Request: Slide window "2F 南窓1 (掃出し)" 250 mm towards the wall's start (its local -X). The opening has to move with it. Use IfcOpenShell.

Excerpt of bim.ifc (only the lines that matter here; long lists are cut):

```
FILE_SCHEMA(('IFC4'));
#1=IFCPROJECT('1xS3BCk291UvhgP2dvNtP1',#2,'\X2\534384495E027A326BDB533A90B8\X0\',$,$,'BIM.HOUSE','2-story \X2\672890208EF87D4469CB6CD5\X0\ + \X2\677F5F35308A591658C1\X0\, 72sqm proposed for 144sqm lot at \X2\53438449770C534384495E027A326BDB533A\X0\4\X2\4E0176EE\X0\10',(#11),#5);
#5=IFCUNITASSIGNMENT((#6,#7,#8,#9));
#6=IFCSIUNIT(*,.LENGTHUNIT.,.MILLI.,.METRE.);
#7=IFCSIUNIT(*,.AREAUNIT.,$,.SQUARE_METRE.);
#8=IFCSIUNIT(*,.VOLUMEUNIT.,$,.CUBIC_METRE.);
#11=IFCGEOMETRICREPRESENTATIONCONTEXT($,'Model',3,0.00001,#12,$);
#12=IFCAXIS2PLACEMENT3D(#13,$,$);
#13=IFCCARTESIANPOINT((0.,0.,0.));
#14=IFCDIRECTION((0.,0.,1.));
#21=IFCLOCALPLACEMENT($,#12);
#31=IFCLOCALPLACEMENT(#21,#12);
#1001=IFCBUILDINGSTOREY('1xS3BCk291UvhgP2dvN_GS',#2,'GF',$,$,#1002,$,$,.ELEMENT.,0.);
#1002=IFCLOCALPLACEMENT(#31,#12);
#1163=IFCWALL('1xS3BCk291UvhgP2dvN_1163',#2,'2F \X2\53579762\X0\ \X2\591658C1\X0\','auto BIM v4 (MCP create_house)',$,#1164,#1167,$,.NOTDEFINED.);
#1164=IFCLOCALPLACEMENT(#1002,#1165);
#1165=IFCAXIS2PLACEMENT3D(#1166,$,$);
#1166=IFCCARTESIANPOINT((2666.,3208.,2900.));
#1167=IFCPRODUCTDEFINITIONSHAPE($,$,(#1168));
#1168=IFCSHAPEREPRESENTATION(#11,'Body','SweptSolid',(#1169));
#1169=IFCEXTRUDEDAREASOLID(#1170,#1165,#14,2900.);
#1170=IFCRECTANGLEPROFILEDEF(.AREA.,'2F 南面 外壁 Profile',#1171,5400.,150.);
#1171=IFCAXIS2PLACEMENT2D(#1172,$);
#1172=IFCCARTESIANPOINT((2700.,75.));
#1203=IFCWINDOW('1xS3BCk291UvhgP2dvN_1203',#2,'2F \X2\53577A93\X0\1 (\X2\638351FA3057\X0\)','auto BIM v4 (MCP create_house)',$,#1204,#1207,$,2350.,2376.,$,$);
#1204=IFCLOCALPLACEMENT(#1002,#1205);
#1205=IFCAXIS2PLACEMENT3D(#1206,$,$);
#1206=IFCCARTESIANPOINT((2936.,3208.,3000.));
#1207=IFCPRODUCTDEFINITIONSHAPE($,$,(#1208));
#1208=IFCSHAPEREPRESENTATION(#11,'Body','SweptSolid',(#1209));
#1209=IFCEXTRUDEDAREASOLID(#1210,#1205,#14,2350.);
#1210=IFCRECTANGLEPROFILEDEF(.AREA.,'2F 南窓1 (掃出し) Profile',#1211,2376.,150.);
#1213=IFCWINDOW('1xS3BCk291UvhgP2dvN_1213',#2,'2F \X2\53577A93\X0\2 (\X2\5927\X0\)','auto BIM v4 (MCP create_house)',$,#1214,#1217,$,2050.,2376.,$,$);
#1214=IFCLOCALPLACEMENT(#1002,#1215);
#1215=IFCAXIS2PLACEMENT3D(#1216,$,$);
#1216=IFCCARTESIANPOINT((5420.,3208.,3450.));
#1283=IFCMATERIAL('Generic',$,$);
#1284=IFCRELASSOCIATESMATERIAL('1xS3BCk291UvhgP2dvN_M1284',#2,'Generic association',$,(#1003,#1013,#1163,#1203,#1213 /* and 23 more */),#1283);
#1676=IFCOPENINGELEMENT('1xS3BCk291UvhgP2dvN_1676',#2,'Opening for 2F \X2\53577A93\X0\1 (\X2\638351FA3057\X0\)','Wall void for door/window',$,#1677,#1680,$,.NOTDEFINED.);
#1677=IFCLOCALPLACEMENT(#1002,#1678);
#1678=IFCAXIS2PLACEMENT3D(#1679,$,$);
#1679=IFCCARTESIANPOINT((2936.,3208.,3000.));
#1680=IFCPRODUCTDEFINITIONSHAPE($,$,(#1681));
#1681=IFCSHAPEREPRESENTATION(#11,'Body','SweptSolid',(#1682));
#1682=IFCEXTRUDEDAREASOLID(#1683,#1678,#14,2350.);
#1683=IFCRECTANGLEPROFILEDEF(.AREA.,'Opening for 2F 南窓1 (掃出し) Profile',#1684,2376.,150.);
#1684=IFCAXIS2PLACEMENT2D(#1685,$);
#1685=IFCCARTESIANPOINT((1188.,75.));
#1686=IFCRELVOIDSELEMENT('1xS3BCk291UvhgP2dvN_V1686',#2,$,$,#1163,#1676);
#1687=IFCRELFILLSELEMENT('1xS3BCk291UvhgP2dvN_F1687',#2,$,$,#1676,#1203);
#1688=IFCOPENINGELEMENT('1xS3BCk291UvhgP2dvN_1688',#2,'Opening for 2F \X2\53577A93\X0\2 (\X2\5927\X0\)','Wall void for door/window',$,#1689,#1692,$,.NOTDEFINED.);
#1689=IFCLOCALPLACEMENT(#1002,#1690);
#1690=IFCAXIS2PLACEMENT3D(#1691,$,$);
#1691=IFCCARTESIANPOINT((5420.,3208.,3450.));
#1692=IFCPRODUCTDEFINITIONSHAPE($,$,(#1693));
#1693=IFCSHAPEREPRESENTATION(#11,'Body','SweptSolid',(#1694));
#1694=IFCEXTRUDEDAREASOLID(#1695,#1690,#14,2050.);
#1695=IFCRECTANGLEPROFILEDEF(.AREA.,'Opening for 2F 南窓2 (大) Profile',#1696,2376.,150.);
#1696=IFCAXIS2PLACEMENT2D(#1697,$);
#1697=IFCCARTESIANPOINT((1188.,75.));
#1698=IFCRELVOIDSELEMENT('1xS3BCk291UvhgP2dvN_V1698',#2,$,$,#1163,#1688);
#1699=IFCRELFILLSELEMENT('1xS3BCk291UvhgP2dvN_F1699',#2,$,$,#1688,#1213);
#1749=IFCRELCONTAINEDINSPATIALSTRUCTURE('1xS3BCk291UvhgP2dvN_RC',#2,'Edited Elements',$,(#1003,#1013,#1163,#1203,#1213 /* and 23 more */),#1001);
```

```python
import ifcopenshell
import ifcopenshell.api.geometry
import ifcopenshell.util.placement

model = ifcopenshell.open("bim.ifc")

window = model.by_guid("1xS3BCk291UvhgP2dvN_1203")
opening = window.FillsVoids[0].RelatingOpeningElement
wall = opening.VoidsElements[0].RelatingBuildingElement

wall_matrix = ifcopenshell.util.placement.get_local_placement(wall.ObjectPlacement)
shift = wall_matrix[:3, 0] * -250.0
before = ifcopenshell.util.placement.get_local_placement(window.ObjectPlacement)[:3, 3].copy()

# The window is not placed relative to its opening, so move both.
for product in (opening, window):
    matrix = ifcopenshell.util.placement.get_local_placement(product.ObjectPlacement)
    matrix[:3, 3] += shift
    ifcopenshell.api.geometry.edit_object_placement(model, product=product, matrix=matrix, is_si=False)

after = ifcopenshell.util.placement.get_local_placement(window.ObjectPlacement)[:3, 3]
print("window moved by", (after - before).round(3) + 0.0)

model.write("bim_updated.ifc")
```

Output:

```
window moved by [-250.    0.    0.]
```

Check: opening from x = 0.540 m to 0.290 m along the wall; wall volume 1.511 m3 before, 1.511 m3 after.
